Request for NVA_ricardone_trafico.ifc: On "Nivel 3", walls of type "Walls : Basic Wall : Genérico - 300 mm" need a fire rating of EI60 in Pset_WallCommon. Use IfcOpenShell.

First a look at what the model holds.

```python
import ifcopenshell
import ifcopenshell.util.element

model = ifcopenshell.open("NVA_ricardone_trafico.ifc")
print(model.schema)
storey = next(s for s in model.by_type("IfcBuildingStorey") if s.Name == "Nivel 3")
walls = [e for e in ifcopenshell.util.element.get_decomposition(storey) if e.is_a("IfcWall")]
seen = {}
for e in walls:
    element_type = ifcopenshell.util.element.get_type(e)
    key = (element_type.Name if element_type != e and element_type else None, ifcopenshell.util.element.get_pset(e, "Pset_WallCommon", "FireRating"))
    seen[key] = seen.get(key, 0) + 1
for (name, value), count in sorted(seen.items(), key=str):
    print(count, "x", name, "|", value)
```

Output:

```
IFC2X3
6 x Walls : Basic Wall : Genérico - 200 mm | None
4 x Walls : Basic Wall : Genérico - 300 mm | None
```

```python
import ifcopenshell
import ifcopenshell.api.pset
import ifcopenshell.util.element

model = ifcopenshell.open("NVA_ricardone_trafico.ifc")

storey = next(s for s in model.by_type("IfcBuildingStorey") if s.Name == "Nivel 3")
walls = [e for e in ifcopenshell.util.element.get_decomposition(storey) if e.is_a("IfcWall")]

count = 0
for e in walls:
    element_type = ifcopenshell.util.element.get_type(e)
    if element_type in (None, e) or element_type.Name != "Walls : Basic Wall : Genérico - 300 mm":
        continue
    # add_pset returns the element's existing set when there is one.
    pset = ifcopenshell.api.pset.add_pset(model, product=e, name="Pset_WallCommon")
    ifcopenshell.api.pset.edit_pset(model, pset=pset, properties={"FireRating": "EI60"})
    count += 1

print(count, "walls updated")

model.write("NVA_ricardone_trafico_v2.ifc")
```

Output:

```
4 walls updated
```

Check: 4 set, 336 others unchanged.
